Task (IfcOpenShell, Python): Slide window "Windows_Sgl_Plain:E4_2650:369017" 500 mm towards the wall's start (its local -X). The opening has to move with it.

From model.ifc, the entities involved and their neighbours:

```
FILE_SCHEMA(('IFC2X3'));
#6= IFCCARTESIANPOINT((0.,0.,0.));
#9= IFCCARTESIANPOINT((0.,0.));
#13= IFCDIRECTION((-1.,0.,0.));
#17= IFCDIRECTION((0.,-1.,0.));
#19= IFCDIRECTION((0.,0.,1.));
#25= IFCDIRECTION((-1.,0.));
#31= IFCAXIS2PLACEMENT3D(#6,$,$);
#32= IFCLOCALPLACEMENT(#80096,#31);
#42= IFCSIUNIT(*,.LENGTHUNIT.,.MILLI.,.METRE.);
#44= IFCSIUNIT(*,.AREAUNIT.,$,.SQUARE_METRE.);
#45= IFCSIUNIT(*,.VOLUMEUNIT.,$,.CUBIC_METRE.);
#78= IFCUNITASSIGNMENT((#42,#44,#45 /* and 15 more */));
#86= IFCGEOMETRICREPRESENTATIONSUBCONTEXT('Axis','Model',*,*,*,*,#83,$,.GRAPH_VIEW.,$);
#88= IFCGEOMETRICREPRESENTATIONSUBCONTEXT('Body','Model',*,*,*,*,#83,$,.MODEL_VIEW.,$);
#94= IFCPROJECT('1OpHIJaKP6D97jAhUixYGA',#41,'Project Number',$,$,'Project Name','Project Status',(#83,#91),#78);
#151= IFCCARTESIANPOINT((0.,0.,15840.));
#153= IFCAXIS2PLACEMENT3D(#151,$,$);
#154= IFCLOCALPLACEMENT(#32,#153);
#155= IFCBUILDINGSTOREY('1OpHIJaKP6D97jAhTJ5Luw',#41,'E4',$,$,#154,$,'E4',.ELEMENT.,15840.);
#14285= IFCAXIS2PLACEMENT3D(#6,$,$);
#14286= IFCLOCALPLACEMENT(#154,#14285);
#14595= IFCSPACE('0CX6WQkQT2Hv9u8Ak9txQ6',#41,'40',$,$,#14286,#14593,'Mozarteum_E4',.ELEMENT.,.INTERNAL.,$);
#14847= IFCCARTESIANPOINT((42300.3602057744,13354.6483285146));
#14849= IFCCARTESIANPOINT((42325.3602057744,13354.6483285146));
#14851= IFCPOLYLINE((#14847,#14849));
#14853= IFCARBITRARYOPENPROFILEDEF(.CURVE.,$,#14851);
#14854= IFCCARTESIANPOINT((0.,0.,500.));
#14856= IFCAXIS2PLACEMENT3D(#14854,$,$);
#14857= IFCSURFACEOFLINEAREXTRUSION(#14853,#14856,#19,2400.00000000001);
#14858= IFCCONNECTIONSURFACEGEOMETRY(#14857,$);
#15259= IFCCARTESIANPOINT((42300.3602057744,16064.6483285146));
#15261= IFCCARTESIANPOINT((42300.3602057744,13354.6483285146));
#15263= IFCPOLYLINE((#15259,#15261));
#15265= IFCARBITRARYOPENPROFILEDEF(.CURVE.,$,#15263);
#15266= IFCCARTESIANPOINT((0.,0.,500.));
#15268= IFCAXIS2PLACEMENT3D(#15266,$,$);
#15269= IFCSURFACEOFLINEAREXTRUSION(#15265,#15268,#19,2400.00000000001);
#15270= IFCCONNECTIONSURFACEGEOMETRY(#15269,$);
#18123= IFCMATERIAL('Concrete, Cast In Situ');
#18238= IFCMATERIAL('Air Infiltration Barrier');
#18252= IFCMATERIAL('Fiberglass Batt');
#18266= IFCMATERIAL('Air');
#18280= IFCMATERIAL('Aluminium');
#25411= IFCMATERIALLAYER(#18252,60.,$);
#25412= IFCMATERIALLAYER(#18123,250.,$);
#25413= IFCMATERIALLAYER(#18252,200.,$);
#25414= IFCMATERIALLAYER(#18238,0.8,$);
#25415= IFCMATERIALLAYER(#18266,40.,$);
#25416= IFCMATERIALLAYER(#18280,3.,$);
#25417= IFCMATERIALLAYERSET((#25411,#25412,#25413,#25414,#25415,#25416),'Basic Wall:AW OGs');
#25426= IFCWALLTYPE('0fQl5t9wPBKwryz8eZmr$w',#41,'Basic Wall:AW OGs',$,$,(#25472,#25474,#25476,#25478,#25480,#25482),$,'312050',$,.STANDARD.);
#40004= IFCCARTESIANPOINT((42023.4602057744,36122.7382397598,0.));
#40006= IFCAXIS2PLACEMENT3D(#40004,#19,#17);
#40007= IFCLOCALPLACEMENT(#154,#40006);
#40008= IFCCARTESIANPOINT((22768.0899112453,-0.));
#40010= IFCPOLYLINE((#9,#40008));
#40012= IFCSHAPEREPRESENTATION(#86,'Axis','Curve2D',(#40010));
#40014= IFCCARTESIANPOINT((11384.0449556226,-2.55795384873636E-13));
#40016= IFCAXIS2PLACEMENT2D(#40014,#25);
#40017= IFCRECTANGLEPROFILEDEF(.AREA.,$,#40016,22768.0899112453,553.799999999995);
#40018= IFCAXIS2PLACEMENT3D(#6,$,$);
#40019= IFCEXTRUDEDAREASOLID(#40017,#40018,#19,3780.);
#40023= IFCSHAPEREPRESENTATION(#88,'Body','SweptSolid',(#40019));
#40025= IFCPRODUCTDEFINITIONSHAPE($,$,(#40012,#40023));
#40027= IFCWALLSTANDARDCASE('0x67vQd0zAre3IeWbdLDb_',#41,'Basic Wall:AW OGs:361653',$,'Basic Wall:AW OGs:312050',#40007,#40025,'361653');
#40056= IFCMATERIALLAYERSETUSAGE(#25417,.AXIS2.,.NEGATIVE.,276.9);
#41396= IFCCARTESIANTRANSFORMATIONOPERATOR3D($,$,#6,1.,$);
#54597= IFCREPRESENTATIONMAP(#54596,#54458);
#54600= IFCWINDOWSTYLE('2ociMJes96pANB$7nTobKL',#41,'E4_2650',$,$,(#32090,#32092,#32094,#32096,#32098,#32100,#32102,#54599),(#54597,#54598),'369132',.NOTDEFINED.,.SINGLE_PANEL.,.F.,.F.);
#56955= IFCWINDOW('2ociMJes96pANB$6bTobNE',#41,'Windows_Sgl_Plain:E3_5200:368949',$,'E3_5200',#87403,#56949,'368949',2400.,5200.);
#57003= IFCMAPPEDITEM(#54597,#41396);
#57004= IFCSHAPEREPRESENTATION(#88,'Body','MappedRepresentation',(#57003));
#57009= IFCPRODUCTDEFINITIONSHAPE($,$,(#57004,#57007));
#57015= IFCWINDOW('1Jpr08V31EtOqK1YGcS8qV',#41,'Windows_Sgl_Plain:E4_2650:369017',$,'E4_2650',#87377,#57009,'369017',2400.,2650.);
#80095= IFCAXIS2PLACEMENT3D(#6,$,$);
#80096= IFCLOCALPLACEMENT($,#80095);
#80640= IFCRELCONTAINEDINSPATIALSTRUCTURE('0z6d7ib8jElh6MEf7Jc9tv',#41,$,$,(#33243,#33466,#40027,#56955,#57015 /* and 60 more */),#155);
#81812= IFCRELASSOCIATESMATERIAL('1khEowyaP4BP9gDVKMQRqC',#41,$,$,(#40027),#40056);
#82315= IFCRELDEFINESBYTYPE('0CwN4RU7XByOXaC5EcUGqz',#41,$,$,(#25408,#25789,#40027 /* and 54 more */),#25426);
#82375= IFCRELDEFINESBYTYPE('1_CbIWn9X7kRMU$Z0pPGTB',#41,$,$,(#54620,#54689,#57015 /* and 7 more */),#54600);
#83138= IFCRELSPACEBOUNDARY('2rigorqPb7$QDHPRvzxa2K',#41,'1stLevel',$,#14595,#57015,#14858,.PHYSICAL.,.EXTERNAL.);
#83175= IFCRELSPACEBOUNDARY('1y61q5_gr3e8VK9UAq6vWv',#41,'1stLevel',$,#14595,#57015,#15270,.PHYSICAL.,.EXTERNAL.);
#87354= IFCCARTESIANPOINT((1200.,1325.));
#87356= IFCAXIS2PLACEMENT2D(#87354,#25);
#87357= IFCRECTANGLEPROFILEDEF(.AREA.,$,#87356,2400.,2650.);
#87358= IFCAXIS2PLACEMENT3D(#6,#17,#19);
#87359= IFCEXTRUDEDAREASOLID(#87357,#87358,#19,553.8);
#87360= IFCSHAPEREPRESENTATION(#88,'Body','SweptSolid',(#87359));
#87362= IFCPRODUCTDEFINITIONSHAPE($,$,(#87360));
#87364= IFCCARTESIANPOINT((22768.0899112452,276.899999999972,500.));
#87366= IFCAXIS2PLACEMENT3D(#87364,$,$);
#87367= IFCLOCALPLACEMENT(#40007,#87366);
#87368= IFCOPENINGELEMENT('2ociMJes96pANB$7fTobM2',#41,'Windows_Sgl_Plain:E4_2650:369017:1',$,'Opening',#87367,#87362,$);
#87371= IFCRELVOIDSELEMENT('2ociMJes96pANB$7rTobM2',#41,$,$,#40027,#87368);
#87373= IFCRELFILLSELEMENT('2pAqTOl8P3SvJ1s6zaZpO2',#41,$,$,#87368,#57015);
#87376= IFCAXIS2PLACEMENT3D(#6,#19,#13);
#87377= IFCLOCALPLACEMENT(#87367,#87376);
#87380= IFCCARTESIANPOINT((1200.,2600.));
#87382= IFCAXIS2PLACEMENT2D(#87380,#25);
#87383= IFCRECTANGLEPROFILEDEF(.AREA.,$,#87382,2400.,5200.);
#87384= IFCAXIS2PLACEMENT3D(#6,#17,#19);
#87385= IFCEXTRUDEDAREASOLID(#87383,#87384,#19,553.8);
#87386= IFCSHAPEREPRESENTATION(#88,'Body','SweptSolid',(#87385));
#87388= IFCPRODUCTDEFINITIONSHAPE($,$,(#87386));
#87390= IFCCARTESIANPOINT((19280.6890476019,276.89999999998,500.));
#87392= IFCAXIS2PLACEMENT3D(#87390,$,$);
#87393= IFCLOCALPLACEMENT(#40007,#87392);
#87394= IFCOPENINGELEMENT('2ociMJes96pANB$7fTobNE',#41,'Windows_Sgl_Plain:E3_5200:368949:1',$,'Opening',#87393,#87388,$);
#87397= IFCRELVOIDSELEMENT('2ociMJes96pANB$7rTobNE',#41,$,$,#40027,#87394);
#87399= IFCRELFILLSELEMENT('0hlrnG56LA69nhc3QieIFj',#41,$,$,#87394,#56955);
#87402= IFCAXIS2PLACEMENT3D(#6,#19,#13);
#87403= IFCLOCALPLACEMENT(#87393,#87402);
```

```python
import numpy as np
import ifcopenshell
import ifcopenshell.api.geometry
import ifcopenshell.util.placement
import ifcopenshell.util.unit

model = ifcopenshell.open("model.ifc")
unit_scale = ifcopenshell.util.unit.calculate_unit_scale(model)

window = model.by_id(57015)
opening = window.FillsVoids[0].RelatingOpeningElement
wall = opening.VoidsElements[0].RelatingBuildingElement

wall_matrix = ifcopenshell.util.placement.get_local_placement(wall.ObjectPlacement)
shift = wall_matrix[:3, 0] * -0.5 / unit_scale
before = ifcopenshell.util.placement.get_local_placement(window.ObjectPlacement)[:3, 3].copy()

# The window is placed relative to its opening, so it follows when the opening moves.
matrix = ifcopenshell.util.placement.get_local_placement(opening.ObjectPlacement)
matrix[:3, 3] += shift
ifcopenshell.api.geometry.edit_object_placement(
    model, product=opening, matrix=matrix, is_si=False, should_transform_children=True
)

# Space boundary surfaces are stored in each space's coordinates; move them too.
for rel in window.ProvidesBoundaries:
    if not rel.ConnectionGeometry:
        continue
    surface = rel.ConnectionGeometry.SurfaceOnRelatingElement
    space_matrix = ifcopenshell.util.placement.get_local_placement(rel.RelatingSpace.ObjectPlacement)
    point = np.array(surface.Position.Location.Coordinates) + space_matrix[:3, :3].T @ shift
    surface.Position = model.createIfcAxis2Placement3D(
        model.createIfcCartesianPoint(point.tolist()), surface.Position.Axis, surface.Position.RefDirection
    )

after = ifcopenshell.util.placement.get_local_placement(window.ObjectPlacement)[:3, 3]
print("window moved by", (after - before).round(3) + 0.0)

model.write("model_rev.ifc")
```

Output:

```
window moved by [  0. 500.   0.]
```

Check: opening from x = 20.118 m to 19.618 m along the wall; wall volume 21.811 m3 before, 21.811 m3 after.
